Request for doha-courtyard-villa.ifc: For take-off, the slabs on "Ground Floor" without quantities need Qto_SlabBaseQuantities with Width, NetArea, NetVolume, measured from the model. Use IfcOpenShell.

First a look at what the model holds.

```python
import ifcopenshell
import ifcopenshell.util.element
import ifcopenshell.util.unit

model = ifcopenshell.open("doha-courtyard-villa.ifc")
print(model.schema)
for unit_type in ("LENGTHUNIT", "AREAUNIT", "VOLUMEUNIT"):
    print(unit_type, ifcopenshell.util.unit.calculate_unit_scale(model, unit_type))
storey = next(s for s in model.by_type("IfcBuildingStorey") if s.Name == "Ground Floor")
slabs = [e for e in ifcopenshell.util.element.get_decomposition(storey) if e.is_a("IfcSlab")]
for e in sorted(slabs, key=lambda e: e.id()):
    print(e.id(), e.is_a(), e.Name, list(ifcopenshell.util.element.get_psets(e, qtos_only=True)), sep=" | ")
```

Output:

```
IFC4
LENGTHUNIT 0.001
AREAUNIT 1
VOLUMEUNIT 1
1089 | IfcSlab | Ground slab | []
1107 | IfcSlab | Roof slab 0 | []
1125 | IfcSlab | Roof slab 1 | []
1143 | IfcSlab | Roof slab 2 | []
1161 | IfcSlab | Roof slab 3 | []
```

```python
import ifcopenshell
import ifcopenshell.api.pset
import ifcopenshell.geom
import ifcopenshell.util.element
import ifcopenshell.util.shape
import ifcopenshell.util.unit

model = ifcopenshell.open("doha-courtyard-villa.ifc")
unit_scale = ifcopenshell.util.unit.calculate_unit_scale(model)
area_scale = ifcopenshell.util.unit.calculate_unit_scale(model, "AREAUNIT")
volume_scale = ifcopenshell.util.unit.calculate_unit_scale(model, "VOLUMEUNIT")
settings = ifcopenshell.geom.settings()

storey = next(s for s in model.by_type("IfcBuildingStorey") if s.Name == "Ground Floor")
slabs = [e for e in ifcopenshell.util.element.get_decomposition(storey) if e.is_a("IfcSlab")]

for e in sorted(slabs, key=lambda e: e.id()):
    if ifcopenshell.util.element.get_psets(e, qtos_only=True, should_inherit=False):
        continue
    # Geometry comes back in metres, in the element's own axes.
    shape = ifcopenshell.geom.create_shape(settings, e)
    values = {
        "Width": ifcopenshell.util.shape.get_z(shape.geometry) / unit_scale,
        "NetArea": ifcopenshell.util.shape.get_footprint_area(shape.geometry) / area_scale,
        "NetVolume": ifcopenshell.util.shape.get_volume(shape.geometry) / volume_scale,
    }
    qto = ifcopenshell.api.pset.add_qto(model, product=e, name="Qto_SlabBaseQuantities")
    ifcopenshell.api.pset.edit_qto(model, qto=qto, properties=values)
    print(e.id(), {k: round(v, 3) for k, v in values.items()})

model.write("doha-courtyard-villa-out.ifc")
```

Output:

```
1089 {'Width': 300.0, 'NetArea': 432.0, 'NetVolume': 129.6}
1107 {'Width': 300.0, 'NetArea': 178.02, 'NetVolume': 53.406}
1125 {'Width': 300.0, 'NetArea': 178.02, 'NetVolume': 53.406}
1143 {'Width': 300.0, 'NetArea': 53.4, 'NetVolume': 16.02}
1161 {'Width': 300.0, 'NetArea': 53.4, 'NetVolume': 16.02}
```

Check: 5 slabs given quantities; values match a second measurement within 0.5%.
